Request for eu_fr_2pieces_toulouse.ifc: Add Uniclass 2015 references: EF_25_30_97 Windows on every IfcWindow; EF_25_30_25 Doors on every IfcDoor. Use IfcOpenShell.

First a look at what the model holds.

```python
import ifcopenshell

model = ifcopenshell.open("eu_fr_2pieces_toulouse.ifc")
print(model.schema)
print("classifications:", [c.Name for c in model.by_type("IfcClassification")])
for ifc_class in ("IfcDoor", "IfcRoof", "IfcStair", "IfcWall", "IfcWindow"):
    print(ifc_class, len(model.by_type(ifc_class)))
```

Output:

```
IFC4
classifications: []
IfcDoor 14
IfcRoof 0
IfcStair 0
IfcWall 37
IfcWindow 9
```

```python
import ifcopenshell
import ifcopenshell.api.classification

model = ifcopenshell.open("eu_fr_2pieces_toulouse.ifc")

system = ifcopenshell.api.classification.add_classification(model, classification="Uniclass 2015")

codes = {
    "IfcWindow": ("EF_25_30_97", "Windows"),
    "IfcDoor": ("EF_25_30_25", "Doors"),
}
for ifc_class, (code, name) in codes.items():
    products = model.by_type(ifc_class)
    ifcopenshell.api.classification.add_reference(
        model, products=products, classification=system, identification=code, name=name
    )
    print(code, len(products))

model.write("eu_fr_2pieces_toulouse_edited.ifc")
```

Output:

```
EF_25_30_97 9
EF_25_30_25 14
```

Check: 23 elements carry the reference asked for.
